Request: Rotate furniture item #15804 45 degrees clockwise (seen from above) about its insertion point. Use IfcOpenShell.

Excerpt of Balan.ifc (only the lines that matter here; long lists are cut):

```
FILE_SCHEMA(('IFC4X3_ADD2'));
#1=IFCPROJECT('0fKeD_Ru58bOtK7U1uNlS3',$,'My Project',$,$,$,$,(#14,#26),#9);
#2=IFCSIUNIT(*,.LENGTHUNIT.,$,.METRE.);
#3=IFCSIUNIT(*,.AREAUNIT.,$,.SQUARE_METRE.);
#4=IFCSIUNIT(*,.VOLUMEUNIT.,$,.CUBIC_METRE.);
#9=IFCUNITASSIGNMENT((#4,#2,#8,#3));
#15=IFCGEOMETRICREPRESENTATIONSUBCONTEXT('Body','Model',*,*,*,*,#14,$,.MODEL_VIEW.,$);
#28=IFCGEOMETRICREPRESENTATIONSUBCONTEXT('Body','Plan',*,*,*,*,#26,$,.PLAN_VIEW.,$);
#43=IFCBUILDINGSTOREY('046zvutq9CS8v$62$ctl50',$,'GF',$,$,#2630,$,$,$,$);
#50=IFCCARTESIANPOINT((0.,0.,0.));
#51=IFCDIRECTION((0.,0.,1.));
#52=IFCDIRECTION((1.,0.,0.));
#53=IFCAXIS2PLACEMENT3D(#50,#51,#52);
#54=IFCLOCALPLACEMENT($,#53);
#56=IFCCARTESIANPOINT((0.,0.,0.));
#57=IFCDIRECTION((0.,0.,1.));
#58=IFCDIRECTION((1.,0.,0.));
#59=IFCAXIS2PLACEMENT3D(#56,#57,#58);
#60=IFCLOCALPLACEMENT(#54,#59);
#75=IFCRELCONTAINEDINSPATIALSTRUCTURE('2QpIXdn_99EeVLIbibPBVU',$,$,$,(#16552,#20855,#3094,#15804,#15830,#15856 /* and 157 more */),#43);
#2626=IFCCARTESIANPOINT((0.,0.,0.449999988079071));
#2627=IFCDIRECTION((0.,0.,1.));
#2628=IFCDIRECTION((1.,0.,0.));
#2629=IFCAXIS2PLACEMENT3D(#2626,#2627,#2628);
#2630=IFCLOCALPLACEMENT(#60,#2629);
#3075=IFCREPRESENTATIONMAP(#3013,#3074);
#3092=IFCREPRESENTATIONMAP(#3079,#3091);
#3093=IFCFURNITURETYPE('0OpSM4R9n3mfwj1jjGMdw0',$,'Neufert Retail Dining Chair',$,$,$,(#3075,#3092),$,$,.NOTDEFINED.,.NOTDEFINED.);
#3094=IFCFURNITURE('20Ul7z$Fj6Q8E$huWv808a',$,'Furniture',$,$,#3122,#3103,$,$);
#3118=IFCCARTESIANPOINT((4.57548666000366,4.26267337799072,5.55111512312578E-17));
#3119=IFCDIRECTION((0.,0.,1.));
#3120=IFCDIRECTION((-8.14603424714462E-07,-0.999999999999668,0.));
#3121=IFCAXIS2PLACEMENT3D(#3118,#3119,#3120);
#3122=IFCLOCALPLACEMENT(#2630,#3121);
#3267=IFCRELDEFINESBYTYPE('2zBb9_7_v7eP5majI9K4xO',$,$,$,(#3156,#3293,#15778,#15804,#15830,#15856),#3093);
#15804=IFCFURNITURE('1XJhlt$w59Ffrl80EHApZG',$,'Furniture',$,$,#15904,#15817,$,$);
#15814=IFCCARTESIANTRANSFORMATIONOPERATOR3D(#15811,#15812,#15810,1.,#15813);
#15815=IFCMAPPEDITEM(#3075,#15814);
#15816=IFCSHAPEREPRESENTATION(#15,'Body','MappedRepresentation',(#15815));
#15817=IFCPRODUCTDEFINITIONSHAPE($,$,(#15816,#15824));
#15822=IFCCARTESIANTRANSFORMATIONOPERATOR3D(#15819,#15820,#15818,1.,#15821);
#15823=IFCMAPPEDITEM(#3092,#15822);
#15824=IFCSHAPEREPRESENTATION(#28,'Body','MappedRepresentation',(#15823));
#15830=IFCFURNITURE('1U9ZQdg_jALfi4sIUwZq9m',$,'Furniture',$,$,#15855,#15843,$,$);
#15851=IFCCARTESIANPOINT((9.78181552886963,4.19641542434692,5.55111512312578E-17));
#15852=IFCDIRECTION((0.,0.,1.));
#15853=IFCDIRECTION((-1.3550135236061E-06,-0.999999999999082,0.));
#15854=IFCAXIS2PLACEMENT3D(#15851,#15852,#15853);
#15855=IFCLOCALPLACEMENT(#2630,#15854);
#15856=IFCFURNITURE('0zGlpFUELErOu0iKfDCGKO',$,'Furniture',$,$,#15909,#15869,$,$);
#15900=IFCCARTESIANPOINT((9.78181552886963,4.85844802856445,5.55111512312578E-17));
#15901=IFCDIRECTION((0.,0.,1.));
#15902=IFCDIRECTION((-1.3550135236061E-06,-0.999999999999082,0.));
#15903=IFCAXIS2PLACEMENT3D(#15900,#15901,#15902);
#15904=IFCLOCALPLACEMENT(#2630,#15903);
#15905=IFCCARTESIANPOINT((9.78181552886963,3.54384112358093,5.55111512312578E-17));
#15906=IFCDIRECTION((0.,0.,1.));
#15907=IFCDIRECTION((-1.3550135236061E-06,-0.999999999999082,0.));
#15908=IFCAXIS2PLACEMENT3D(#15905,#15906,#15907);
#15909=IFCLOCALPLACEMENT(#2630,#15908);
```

```python
import ifcopenshell
import ifcopenshell.api.geometry
import ifcopenshell.util.placement

model = ifcopenshell.open("Balan.ifc")

item = model.by_guid("1XJhlt$w59Ffrl80EHApZG")
matrix = ifcopenshell.util.placement.get_local_placement(item.ObjectPlacement)
matrix = matrix @ ifcopenshell.util.placement.rotation(-45, "Z")
ifcopenshell.api.geometry.edit_object_placement(model, product=item, matrix=matrix, is_si=False)

print(ifcopenshell.util.placement.get_local_placement(item.ObjectPlacement).round(3) + 0.0)

model.write("Balan_v2.ifc")
```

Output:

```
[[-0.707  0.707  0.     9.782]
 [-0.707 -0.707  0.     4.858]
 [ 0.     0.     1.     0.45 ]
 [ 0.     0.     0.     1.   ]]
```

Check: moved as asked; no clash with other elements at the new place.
